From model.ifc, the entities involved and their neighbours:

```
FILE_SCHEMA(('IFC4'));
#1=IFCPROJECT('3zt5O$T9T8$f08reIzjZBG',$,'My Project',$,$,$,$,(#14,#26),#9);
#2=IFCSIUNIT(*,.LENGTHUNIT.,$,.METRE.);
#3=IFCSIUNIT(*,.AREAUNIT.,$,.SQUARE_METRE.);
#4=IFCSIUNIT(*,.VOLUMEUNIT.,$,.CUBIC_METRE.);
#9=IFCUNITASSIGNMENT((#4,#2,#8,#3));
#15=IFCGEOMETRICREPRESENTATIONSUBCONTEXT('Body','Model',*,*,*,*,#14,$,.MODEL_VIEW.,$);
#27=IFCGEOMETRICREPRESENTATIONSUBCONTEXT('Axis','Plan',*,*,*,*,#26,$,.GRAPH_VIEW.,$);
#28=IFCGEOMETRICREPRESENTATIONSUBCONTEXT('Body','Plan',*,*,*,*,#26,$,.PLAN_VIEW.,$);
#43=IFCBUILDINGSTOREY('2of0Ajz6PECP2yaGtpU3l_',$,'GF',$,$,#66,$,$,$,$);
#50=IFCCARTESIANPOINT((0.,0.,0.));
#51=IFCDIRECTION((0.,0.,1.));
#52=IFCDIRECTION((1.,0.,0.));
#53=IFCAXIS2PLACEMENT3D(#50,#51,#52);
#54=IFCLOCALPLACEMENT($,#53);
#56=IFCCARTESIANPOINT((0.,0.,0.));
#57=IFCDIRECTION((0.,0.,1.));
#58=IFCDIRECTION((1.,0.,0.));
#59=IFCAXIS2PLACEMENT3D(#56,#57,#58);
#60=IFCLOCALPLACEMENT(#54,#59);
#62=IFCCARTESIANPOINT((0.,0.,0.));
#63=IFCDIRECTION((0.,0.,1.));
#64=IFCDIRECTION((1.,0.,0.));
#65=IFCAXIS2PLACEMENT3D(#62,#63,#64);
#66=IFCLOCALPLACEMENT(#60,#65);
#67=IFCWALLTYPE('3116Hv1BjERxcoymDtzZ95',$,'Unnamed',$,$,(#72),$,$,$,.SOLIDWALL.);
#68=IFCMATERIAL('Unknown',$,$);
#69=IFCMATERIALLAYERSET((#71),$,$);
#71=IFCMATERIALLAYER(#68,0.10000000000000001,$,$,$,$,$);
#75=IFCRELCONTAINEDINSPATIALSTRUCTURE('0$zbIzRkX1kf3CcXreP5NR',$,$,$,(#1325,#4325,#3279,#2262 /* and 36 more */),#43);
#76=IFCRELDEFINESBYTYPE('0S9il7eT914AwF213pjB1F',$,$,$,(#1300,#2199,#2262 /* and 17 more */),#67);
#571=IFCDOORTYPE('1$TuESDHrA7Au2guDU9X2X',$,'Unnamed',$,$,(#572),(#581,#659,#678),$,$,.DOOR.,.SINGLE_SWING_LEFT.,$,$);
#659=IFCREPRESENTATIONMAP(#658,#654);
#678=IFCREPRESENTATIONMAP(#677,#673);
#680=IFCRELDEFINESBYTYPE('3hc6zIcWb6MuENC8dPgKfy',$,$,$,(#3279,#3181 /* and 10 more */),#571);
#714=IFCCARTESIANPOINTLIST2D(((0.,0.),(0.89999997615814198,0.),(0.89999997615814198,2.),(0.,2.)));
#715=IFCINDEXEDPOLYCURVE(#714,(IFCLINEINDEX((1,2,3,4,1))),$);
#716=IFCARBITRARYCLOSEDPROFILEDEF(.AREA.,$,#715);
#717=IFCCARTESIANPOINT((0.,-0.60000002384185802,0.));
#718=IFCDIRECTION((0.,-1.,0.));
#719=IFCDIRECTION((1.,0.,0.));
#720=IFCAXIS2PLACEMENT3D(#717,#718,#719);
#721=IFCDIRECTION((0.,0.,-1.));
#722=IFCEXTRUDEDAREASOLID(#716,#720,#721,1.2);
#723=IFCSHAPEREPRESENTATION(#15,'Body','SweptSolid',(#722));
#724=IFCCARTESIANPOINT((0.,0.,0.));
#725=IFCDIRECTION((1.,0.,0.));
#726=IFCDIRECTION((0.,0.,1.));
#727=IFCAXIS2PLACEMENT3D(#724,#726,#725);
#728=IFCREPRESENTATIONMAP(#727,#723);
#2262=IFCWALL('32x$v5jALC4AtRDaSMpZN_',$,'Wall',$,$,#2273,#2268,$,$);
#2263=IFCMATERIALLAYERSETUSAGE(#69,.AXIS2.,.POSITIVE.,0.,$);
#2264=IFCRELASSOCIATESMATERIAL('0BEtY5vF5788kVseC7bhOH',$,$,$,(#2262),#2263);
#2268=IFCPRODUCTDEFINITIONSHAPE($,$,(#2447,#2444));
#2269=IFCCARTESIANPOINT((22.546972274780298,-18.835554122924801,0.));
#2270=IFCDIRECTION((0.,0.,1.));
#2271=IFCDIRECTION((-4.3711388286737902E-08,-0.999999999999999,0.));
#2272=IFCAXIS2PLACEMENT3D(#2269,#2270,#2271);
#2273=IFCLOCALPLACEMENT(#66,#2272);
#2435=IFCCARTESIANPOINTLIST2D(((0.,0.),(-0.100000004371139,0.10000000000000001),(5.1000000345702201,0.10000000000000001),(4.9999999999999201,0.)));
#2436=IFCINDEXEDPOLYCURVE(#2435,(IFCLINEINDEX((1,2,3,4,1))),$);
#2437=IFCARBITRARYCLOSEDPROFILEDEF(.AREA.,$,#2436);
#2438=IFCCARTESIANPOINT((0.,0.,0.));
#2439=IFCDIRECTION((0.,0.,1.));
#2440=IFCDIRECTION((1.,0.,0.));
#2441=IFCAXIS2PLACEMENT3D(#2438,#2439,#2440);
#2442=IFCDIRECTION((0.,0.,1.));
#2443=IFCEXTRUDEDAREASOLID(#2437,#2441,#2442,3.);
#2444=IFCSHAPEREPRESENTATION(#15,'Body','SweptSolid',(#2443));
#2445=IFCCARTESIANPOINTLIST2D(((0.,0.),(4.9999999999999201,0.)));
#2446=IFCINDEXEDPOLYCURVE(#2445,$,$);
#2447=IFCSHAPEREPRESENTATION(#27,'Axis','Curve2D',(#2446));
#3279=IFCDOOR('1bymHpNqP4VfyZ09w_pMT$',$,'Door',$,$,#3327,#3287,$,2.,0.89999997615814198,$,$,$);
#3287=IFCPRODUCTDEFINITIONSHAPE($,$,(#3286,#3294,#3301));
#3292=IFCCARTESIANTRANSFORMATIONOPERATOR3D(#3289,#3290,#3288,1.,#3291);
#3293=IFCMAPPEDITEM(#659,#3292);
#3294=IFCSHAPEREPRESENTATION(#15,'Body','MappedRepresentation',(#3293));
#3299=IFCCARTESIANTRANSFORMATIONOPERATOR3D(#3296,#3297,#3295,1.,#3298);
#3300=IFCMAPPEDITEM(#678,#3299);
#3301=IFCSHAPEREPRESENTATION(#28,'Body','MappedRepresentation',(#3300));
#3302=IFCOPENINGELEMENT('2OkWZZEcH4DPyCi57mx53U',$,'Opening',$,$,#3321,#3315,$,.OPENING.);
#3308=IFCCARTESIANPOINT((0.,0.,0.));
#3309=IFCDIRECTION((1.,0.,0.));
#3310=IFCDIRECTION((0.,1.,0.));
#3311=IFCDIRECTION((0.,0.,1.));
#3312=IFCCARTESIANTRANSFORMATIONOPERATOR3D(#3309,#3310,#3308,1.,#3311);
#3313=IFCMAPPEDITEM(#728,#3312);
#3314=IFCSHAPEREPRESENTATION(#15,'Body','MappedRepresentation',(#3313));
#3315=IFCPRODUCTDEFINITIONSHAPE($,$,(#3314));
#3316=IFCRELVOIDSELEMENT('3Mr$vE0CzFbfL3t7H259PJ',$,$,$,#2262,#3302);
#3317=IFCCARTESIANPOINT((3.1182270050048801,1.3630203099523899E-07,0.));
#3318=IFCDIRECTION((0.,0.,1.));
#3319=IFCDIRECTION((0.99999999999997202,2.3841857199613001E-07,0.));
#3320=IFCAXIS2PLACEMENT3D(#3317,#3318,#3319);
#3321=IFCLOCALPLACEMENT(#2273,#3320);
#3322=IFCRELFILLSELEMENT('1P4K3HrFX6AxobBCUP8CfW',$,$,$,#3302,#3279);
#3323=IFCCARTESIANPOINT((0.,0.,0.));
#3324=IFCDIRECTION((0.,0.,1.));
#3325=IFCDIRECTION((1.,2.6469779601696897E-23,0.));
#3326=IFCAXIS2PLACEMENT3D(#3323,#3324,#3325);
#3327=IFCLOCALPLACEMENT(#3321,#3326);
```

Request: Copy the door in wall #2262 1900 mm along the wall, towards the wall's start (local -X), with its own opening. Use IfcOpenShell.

```python
import ifcopenshell
import ifcopenshell.api.feature
import ifcopenshell.api.geometry
import ifcopenshell.api.root
import ifcopenshell.geom
import ifcopenshell.util.element
import ifcopenshell.util.placement
import ifcopenshell.util.shape
import ifcopenshell.util.unit

model = ifcopenshell.open("model.ifc")
unit_scale = ifcopenshell.util.unit.calculate_unit_scale(model)
settings = ifcopenshell.geom.settings()


def volume(element):
    """Net volume in cubic metres, openings subtracted."""
    shape = ifcopenshell.geom.create_shape(settings, element)
    return ifcopenshell.util.shape.get_volume(shape.geometry)


door = model.by_guid("1bymHpNqP4VfyZ09w_pMT$")
opening = door.FillsVoids[0].RelatingOpeningElement
wall = opening.VoidsElements[0].RelatingBuildingElement
before = volume(wall)
shift = ifcopenshell.util.placement.get_local_placement(wall.ObjectPlacement)[:3, 0] * -1.9 / unit_scale

# copy_class copies the void relationship, type, container and properties, but no geometry.
new_opening = ifcopenshell.api.root.copy_class(model, product=opening)
new_opening.Representation = ifcopenshell.util.element.copy_deep(
    model, opening.Representation, exclude=["IfcGeometricRepresentationContext", "IfcRepresentationMap"]
)
new_door = ifcopenshell.api.root.copy_class(model, product=door)
new_door.Representation = ifcopenshell.util.element.copy_deep(
    model, door.Representation, exclude=["IfcGeometricRepresentationContext", "IfcRepresentationMap"]
)
ifcopenshell.api.feature.add_filling(model, opening=new_opening, element=new_door)

for old, new in ((opening, new_opening), (door, new_door)):
    matrix = ifcopenshell.util.placement.get_local_placement(old.ObjectPlacement)
    matrix[:3, 3] += shift
    ifcopenshell.api.geometry.edit_object_placement(model, product=new, matrix=matrix, is_si=False)

after = volume(wall)

print(f"wall volume {before:.3f} -> {after:.3f} m3")

model.write("model-out.ifc")
```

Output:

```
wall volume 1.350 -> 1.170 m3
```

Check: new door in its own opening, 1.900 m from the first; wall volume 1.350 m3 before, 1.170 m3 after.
